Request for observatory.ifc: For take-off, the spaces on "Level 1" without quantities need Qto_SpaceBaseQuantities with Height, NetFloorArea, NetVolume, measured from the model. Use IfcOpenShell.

First a look at what the model holds.

```python
import ifcopenshell
import ifcopenshell.util.element
import ifcopenshell.util.unit

model = ifcopenshell.open("observatory.ifc")
print(model.schema)
for unit_type in ("LENGTHUNIT", "AREAUNIT", "VOLUMEUNIT"):
    print(unit_type, ifcopenshell.util.unit.calculate_unit_scale(model, unit_type))
storey = next(s for s in model.by_type("IfcBuildingStorey") if s.Name == "Level 1")
spaces = [e for e in ifcopenshell.util.element.get_decomposition(storey) if e.is_a("IfcSpace")]
for e in sorted(spaces, key=lambda e: e.id()):
    print(e.id(), e.is_a(), e.Name, list(ifcopenshell.util.element.get_psets(e, qtos_only=True)), sep=" | ")
```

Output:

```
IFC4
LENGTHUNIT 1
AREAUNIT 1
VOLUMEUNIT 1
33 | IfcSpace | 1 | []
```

```python
import ifcopenshell
import ifcopenshell.api.pset
import ifcopenshell.geom
import ifcopenshell.util.element
import ifcopenshell.util.shape
import ifcopenshell.util.unit

model = ifcopenshell.open("observatory.ifc")
unit_scale = ifcopenshell.util.unit.calculate_unit_scale(model)
area_scale = ifcopenshell.util.unit.calculate_unit_scale(model, "AREAUNIT")
volume_scale = ifcopenshell.util.unit.calculate_unit_scale(model, "VOLUMEUNIT")
settings = ifcopenshell.geom.settings()

storey = next(s for s in model.by_type("IfcBuildingStorey") if s.Name == "Level 1")
spaces = [e for e in ifcopenshell.util.element.get_decomposition(storey) if e.is_a("IfcSpace")]

for e in sorted(spaces, key=lambda e: e.id()):
    if ifcopenshell.util.element.get_psets(e, qtos_only=True, should_inherit=False):
        continue
    # Geometry comes back in metres, in the element's own axes.
    shape = ifcopenshell.geom.create_shape(settings, e)
    values = {
        "Height": ifcopenshell.util.shape.get_z(shape.geometry) / unit_scale,
        "NetFloorArea": ifcopenshell.util.shape.get_footprint_area(shape.geometry) / area_scale,
        "NetVolume": ifcopenshell.util.shape.get_volume(shape.geometry) / volume_scale,
    }
    qto = ifcopenshell.api.pset.add_qto(model, product=e, name="Qto_SpaceBaseQuantities")
    ifcopenshell.api.pset.edit_qto(model, qto=qto, properties=values)
    print(e.id(), {k: round(v, 3) for k, v in values.items()})

model.write("observatory_rev.ifc")
```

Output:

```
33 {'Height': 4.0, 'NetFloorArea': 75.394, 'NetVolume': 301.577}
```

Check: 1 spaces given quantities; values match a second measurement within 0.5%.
